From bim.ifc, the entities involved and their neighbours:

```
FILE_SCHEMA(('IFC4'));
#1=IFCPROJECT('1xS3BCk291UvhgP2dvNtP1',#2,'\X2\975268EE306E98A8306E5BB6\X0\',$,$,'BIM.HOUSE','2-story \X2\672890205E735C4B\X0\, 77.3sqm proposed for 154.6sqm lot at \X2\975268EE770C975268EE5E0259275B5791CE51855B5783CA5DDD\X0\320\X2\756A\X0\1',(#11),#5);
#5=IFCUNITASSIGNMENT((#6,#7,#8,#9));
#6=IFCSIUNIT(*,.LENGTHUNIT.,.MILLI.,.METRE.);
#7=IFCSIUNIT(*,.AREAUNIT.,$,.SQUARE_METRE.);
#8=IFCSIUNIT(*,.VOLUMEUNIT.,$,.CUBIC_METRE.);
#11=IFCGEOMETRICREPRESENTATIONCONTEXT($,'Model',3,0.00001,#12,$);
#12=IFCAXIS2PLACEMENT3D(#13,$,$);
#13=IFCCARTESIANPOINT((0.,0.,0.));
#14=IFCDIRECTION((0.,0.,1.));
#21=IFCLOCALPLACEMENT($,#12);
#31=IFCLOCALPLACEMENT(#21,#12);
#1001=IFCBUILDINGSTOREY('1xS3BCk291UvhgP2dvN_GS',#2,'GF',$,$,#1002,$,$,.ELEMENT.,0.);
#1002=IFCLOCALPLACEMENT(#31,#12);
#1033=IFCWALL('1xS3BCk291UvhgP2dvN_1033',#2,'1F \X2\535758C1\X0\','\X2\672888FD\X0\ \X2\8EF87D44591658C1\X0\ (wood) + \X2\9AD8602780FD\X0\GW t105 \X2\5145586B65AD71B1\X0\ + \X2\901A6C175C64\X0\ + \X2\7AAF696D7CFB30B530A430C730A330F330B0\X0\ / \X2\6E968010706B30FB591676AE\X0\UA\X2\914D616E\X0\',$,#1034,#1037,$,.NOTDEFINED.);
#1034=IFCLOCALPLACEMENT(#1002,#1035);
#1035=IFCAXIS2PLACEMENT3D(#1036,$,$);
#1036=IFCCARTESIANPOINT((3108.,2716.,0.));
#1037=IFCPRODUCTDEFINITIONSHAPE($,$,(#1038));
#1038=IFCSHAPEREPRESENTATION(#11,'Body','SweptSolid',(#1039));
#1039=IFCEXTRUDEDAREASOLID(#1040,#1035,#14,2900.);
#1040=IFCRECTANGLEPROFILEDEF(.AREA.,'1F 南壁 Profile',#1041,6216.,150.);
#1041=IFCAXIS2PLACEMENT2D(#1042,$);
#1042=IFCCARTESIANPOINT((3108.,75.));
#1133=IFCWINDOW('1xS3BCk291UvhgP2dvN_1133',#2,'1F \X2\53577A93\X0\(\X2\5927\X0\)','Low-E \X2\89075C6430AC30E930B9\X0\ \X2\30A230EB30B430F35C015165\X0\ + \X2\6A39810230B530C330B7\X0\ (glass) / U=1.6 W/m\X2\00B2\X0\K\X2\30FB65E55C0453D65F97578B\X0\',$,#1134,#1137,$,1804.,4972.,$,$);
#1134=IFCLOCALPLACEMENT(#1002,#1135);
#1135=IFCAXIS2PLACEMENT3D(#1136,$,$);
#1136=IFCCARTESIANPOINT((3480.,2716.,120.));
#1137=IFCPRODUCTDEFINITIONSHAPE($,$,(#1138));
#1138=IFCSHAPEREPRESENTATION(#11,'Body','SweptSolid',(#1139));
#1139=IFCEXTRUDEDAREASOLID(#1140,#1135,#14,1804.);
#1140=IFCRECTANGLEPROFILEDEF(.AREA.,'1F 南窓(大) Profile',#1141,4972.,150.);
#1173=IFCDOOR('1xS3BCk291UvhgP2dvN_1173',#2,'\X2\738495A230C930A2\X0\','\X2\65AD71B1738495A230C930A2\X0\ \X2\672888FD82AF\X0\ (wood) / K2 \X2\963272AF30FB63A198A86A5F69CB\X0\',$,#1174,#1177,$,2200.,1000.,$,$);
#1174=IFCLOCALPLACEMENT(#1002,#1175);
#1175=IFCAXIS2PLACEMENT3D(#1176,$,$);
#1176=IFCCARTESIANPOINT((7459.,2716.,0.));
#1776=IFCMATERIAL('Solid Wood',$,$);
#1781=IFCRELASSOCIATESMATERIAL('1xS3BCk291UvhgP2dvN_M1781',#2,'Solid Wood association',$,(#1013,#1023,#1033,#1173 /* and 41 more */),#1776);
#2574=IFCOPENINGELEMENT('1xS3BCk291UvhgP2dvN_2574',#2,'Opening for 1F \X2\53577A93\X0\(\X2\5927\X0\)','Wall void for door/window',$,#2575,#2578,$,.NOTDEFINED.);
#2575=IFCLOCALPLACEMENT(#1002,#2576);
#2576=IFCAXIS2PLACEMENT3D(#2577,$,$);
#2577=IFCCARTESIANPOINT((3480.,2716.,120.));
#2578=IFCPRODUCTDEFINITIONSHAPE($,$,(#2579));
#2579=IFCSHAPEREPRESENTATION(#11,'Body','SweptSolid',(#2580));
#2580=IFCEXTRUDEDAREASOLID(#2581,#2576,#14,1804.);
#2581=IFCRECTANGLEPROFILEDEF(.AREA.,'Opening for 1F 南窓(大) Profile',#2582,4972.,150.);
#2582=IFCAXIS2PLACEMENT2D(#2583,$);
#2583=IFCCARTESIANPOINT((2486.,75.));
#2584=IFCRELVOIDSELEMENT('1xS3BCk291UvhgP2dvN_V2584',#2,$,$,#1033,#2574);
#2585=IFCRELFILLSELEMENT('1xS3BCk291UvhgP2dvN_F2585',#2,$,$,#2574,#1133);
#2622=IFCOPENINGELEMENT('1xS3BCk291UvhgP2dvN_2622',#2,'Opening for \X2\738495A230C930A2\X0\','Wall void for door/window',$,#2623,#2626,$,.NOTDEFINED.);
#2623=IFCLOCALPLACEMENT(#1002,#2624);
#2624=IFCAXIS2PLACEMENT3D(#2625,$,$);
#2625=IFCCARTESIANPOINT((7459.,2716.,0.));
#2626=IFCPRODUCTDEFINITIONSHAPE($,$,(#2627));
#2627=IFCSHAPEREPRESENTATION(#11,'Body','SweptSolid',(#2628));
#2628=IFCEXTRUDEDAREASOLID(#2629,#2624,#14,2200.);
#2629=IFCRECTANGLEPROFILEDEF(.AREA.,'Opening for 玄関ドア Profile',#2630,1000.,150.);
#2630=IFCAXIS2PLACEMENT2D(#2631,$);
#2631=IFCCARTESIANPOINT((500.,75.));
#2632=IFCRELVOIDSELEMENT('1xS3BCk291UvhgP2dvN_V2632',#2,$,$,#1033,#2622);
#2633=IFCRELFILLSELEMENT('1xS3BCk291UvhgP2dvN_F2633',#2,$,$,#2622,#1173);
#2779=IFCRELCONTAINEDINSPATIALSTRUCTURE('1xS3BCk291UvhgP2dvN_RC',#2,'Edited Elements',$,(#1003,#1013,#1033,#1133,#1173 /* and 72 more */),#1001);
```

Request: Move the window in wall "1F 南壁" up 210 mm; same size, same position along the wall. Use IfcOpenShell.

```python
import numpy as np
import ifcopenshell
import ifcopenshell.api.geometry
import ifcopenshell.util.placement
import ifcopenshell.util.unit

model = ifcopenshell.open("bim.ifc")
unit_scale = ifcopenshell.util.unit.calculate_unit_scale(model)

window = model.by_guid("1xS3BCk291UvhgP2dvN_1133")
opening = window.FillsVoids[0].RelatingOpeningElement
dz = 210.0

shift = np.array([0.0, 0.0, dz])
# The window is not placed relative to its opening, so move both.
for product in (opening, window):
    matrix = ifcopenshell.util.placement.get_local_placement(product.ObjectPlacement)
    matrix[:3, 3] += shift
    ifcopenshell.api.geometry.edit_object_placement(model, product=product, matrix=matrix, is_si=False)

print(f"moved by {dz * unit_scale:+.3f} m")

model.write("bim_rev.ifc")
```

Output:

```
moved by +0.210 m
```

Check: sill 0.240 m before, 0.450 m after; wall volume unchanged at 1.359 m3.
